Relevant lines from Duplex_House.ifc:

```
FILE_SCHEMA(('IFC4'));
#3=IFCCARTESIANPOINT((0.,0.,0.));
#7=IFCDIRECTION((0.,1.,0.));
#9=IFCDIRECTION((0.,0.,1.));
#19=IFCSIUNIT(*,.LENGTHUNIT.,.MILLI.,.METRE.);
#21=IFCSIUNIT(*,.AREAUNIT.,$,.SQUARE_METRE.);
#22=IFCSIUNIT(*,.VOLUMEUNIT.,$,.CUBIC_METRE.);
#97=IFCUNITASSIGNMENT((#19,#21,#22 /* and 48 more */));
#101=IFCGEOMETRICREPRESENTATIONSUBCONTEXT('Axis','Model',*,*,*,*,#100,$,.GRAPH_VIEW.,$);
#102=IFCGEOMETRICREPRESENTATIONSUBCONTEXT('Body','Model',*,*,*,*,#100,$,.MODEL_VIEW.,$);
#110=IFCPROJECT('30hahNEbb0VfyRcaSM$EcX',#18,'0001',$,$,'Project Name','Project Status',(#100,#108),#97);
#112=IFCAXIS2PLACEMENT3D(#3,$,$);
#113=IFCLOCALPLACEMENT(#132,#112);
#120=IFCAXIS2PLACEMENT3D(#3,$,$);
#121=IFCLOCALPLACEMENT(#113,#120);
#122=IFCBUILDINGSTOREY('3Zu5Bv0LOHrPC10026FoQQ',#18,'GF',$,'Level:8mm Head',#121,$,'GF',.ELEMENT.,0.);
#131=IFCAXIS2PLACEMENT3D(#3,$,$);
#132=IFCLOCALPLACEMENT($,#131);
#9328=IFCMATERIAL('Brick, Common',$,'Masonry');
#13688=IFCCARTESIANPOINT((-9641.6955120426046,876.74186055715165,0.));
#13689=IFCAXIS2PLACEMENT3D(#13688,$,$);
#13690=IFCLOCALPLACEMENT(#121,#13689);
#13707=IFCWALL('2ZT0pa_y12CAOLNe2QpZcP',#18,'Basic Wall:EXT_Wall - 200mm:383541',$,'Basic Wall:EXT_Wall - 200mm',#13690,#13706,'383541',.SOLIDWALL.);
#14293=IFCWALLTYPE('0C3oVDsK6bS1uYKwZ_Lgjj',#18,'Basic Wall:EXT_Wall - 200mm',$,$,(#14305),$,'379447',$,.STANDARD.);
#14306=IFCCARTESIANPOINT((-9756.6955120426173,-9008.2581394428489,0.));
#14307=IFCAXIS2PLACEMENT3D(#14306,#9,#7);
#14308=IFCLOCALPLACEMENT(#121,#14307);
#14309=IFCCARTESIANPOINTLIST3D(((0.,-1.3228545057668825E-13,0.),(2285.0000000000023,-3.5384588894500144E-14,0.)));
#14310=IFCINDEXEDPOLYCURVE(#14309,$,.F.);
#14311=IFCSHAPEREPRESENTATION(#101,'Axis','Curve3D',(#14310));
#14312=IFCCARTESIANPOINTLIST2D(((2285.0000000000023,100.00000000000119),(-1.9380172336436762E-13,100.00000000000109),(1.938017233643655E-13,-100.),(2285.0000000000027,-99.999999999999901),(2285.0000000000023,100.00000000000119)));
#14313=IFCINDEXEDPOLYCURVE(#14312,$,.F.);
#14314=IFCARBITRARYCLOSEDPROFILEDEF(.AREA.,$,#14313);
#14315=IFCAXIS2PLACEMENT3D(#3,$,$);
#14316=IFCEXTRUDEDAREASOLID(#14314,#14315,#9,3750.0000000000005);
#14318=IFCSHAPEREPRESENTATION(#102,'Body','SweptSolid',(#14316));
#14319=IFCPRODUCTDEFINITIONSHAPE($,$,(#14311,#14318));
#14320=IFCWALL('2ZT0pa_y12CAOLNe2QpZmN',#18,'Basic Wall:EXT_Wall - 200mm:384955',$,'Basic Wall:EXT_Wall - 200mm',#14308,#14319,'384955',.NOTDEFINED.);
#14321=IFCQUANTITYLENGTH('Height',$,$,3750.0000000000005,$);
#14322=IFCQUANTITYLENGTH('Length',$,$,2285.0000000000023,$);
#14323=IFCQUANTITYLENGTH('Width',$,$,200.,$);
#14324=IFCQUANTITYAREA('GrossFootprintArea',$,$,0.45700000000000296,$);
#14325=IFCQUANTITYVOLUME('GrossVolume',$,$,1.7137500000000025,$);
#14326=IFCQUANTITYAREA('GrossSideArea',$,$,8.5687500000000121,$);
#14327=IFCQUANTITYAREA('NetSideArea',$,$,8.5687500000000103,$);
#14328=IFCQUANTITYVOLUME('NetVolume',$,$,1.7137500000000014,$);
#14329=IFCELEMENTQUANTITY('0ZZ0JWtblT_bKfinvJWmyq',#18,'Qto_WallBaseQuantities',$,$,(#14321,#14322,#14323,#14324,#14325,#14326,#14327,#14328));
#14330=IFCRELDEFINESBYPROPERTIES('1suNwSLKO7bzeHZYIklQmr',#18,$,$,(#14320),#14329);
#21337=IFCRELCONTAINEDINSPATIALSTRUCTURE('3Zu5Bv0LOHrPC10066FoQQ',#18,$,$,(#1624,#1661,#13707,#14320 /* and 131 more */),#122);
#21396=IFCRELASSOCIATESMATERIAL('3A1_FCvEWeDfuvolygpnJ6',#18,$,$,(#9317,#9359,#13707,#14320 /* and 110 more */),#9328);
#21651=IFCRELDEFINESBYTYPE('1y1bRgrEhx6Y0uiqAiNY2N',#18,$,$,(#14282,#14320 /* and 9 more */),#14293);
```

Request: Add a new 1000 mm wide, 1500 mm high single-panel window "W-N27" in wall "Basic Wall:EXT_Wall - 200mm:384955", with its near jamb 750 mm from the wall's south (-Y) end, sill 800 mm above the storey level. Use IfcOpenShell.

```python
import numpy as np
import ifcopenshell
import ifcopenshell.api.feature
import ifcopenshell.api.geometry
import ifcopenshell.api.pset
import ifcopenshell.api.root
import ifcopenshell.api.spatial
import ifcopenshell.geom
import ifcopenshell.util.element
import ifcopenshell.util.placement
import ifcopenshell.util.representation
import ifcopenshell.util.shape
import ifcopenshell.util.unit

model = ifcopenshell.open("Duplex_House.ifc")
unit_scale = ifcopenshell.util.unit.calculate_unit_scale(model)
area_scale = ifcopenshell.util.unit.calculate_unit_scale(model, "AREAUNIT")
volume_scale = ifcopenshell.util.unit.calculate_unit_scale(model, "VOLUMEUNIT")
settings = ifcopenshell.geom.settings()


def volume(element):
    """Net volume in cubic metres, openings subtracted."""
    shape = ifcopenshell.geom.create_shape(settings, element)
    return ifcopenshell.util.shape.get_volume(shape.geometry)


wall = model.by_guid("2ZT0pa_y12CAOLNe2QpZmN")
storey = ifcopenshell.util.element.get_container(wall, ifc_class="IfcBuildingStorey")
context = ifcopenshell.util.representation.get_context(model, "Model", "Body", "MODEL_VIEW")
before = volume(wall)

width, height, from_end, sill = 1, 1.5, 0.75, 0.8  # metres

# The wall runs along its own X axis, and the end named is its -X end.
wall_shape = ifcopenshell.geom.create_shape(settings, wall)
x, y, z = ifcopenshell.util.shape.get_vertices(wall_shape.geometry).T
start = x.min() + from_end
face, thickness = float(y.min()), float(y.max() - y.min())
wall_matrix = ifcopenshell.util.placement.get_local_placement(wall.ObjectPlacement)
level = ifcopenshell.util.placement.get_local_placement(storey.ObjectPlacement)[2, 3]


def in_wall(x, y):
    """Placement at x, y metres in the wall's axes, at sill height."""
    matrix = wall_matrix.copy()
    matrix[:, 3] = wall_matrix @ np.array([x / unit_scale, y / unit_scale, 0.0, 1.0])
    matrix[2, 3] = level + sill / unit_scale
    return matrix


# Opening: a box that overshoots both wall faces by 50 mm.
opening = ifcopenshell.api.root.create_entity(model, ifc_class="IfcOpeningElement", predefined_type="OPENING")
box = ifcopenshell.api.geometry.add_wall_representation(
    model, context=context, length=width, height=height, thickness=thickness + 0.1
)
ifcopenshell.api.geometry.assign_representation(model, product=opening, representation=box)
ifcopenshell.api.geometry.edit_object_placement(model, product=opening, matrix=in_wall(start, face - 0.05), is_si=False)
ifcopenshell.api.feature.add_feature(model, feature=opening, element=wall)

window = ifcopenshell.api.root.create_entity(model, ifc_class="IfcWindow", name="W-N27", predefined_type="WINDOW")
window.OverallWidth, window.OverallHeight = width / unit_scale, height / unit_scale
window.PartitioningType = "SINGLE_PANEL"
body = ifcopenshell.api.geometry.add_window_representation(
    model,
    context=context,
    overall_width=window.OverallWidth,
    overall_height=window.OverallHeight,
    partition_type="SINGLE_PANEL",
)
ifcopenshell.api.geometry.assign_representation(model, product=window, representation=body)
ifcopenshell.api.spatial.assign_container(model, products=[window], relating_structure=storey)
ifcopenshell.api.feature.add_filling(model, opening=opening, element=window)

# Centre the window in the wall's thickness.
ifcopenshell.api.geometry.edit_object_placement(model, product=window, matrix=in_wall(start, face), is_si=False)
window_shape = ifcopenshell.geom.create_shape(settings, window)
depth = ifcopenshell.util.shape.get_vertices(window_shape.geometry)[:, 1]
offset = face + thickness / 2 - (depth.min() + depth.max()) / 2
ifcopenshell.api.geometry.edit_object_placement(model, product=window, matrix=in_wall(start, offset), is_si=False)

after = volume(wall)

# Update the wall's stored quantities.
qto = model.by_id(ifcopenshell.util.element.get_pset(wall, "Qto_WallBaseQuantities", should_inherit=False)["id"])
ifcopenshell.api.pset.edit_qto(model, qto=qto, properties={
    "NetSideArea": after / thickness / area_scale,
    "NetVolume": after / volume_scale,
})

print(f"wall volume {before:.3f} -> {after:.3f} m3")

model.write("Duplex_House_edited.ifc")
```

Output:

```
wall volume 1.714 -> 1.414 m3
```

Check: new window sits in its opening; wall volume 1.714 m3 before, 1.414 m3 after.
